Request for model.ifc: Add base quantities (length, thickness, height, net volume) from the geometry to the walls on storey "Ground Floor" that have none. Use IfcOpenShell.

First a look at what the model holds.

```python
import ifcopenshell
import ifcopenshell.util.element
import ifcopenshell.util.unit

model = ifcopenshell.open("model.ifc")
print(model.schema)
for unit_type in ("LENGTHUNIT", "AREAUNIT", "VOLUMEUNIT"):
    print(unit_type, ifcopenshell.util.unit.calculate_unit_scale(model, unit_type))
storey = next(s for s in model.by_type("IfcBuildingStorey") if s.Name == "Ground Floor")
walls = [e for e in ifcopenshell.util.element.get_decomposition(storey) if e.is_a("IfcWall")]
for e in sorted(walls, key=lambda e: e.id()):
    print(e.id(), e.is_a(), e.Name, list(ifcopenshell.util.element.get_psets(e, qtos_only=True)), sep=" | ")
```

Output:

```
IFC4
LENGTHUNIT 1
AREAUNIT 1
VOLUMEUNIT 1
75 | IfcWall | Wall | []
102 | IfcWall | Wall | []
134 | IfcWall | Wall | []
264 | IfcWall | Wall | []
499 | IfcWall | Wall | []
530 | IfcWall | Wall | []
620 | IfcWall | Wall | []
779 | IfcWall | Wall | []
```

```python
import ifcopenshell
import ifcopenshell.api.pset
import ifcopenshell.geom
import ifcopenshell.util.element
import ifcopenshell.util.shape
import ifcopenshell.util.unit

model = ifcopenshell.open("model.ifc")
unit_scale = ifcopenshell.util.unit.calculate_unit_scale(model)
volume_scale = ifcopenshell.util.unit.calculate_unit_scale(model, "VOLUMEUNIT")
settings = ifcopenshell.geom.settings()

storey = next(s for s in model.by_type("IfcBuildingStorey") if s.Name == "Ground Floor")
walls = [e for e in ifcopenshell.util.element.get_decomposition(storey) if e.is_a("IfcWall")]

for e in sorted(walls, key=lambda e: e.id()):
    if ifcopenshell.util.element.get_psets(e, qtos_only=True, should_inherit=False):
        continue
    # Geometry comes back in metres, in the element's own axes.
    shape = ifcopenshell.geom.create_shape(settings, e)
    values = {
        "Length": ifcopenshell.util.shape.get_x(shape.geometry) / unit_scale,
        "Width": ifcopenshell.util.shape.get_y(shape.geometry) / unit_scale,
        "Height": ifcopenshell.util.shape.get_z(shape.geometry) / unit_scale,
        "NetVolume": ifcopenshell.util.shape.get_volume(shape.geometry) / volume_scale,
    }
    qto = ifcopenshell.api.pset.add_qto(model, product=e, name="Qto_WallBaseQuantities")
    ifcopenshell.api.pset.edit_qto(model, qto=qto, properties=values)
    print(e.id(), {k: round(v, 3) for k, v in values.items()})

model.write("model_v2.ifc")
```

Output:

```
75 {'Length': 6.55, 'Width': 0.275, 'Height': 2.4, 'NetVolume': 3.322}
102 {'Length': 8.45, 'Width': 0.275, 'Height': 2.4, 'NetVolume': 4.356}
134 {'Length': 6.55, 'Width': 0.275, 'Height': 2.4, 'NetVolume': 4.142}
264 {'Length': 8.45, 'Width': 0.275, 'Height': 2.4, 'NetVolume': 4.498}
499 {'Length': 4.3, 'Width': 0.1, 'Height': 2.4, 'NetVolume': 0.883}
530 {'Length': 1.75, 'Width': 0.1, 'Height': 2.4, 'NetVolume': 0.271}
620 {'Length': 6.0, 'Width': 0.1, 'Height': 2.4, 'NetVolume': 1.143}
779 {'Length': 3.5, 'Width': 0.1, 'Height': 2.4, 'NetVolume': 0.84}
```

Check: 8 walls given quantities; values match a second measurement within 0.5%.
